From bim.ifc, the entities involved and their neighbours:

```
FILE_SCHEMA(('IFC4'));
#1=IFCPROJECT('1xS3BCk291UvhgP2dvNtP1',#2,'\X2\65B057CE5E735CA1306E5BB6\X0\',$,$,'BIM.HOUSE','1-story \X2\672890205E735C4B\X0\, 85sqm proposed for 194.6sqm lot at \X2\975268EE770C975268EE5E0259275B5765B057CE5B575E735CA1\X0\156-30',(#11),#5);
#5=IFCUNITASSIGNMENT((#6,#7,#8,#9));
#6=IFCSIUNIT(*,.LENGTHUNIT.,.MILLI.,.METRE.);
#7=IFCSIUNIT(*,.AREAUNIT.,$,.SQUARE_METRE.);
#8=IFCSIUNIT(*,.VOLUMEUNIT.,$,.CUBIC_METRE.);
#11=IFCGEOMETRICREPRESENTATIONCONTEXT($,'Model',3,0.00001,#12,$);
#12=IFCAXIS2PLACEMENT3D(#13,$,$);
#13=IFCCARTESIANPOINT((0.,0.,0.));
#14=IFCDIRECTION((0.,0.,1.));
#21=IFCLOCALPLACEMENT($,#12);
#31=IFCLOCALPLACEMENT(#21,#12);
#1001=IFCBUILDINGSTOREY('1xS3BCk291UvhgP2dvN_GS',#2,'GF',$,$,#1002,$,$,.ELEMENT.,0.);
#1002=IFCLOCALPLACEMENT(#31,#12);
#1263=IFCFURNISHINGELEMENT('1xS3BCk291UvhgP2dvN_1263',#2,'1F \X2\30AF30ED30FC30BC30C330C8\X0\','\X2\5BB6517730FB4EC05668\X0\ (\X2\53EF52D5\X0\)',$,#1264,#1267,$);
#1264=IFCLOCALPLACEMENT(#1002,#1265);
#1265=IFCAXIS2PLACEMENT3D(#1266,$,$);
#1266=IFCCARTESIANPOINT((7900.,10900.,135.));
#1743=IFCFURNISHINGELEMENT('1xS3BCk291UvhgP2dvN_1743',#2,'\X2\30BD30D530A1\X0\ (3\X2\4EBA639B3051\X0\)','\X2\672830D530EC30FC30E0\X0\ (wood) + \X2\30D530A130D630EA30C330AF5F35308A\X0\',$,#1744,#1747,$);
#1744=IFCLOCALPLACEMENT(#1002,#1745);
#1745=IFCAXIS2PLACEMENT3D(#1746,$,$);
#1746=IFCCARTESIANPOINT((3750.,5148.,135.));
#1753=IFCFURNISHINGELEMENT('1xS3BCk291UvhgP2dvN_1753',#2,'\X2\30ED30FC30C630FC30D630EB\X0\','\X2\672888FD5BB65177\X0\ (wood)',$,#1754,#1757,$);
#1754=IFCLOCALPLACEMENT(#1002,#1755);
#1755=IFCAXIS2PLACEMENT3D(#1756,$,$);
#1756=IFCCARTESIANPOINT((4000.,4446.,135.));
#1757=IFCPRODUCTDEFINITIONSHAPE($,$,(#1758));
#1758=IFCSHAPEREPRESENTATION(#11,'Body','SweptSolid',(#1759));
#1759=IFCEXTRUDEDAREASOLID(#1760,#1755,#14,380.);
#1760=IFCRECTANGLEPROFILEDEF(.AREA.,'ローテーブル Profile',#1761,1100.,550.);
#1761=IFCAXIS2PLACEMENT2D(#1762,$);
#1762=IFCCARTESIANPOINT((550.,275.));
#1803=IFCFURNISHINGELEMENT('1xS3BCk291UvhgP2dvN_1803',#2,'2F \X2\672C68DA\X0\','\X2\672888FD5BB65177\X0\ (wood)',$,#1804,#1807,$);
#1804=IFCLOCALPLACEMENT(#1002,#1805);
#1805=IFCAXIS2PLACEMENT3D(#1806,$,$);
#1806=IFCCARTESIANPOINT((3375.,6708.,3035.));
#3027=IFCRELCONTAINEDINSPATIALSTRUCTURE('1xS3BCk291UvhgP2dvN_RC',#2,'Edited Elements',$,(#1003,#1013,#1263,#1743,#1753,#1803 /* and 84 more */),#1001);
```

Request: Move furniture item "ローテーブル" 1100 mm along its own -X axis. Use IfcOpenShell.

```python
import ifcopenshell
import ifcopenshell.api.geometry
import ifcopenshell.util.placement
import ifcopenshell.util.unit

model = ifcopenshell.open("bim.ifc")
unit_scale = ifcopenshell.util.unit.calculate_unit_scale(model)

item = model.by_guid("1xS3BCk291UvhgP2dvN_1753")
matrix = ifcopenshell.util.placement.get_local_placement(item.ObjectPlacement)
matrix[:3, 3] -= matrix[:3, 0] * 1.1 / unit_scale
ifcopenshell.api.geometry.edit_object_placement(model, product=item, matrix=matrix, is_si=False)

print(ifcopenshell.util.placement.get_local_placement(item.ObjectPlacement).round(3) + 0.0)

model.write("bim-out.ifc")
```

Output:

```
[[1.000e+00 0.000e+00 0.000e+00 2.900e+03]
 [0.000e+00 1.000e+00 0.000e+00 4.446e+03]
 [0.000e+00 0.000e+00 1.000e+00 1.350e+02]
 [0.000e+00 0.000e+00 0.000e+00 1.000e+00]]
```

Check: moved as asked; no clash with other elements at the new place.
